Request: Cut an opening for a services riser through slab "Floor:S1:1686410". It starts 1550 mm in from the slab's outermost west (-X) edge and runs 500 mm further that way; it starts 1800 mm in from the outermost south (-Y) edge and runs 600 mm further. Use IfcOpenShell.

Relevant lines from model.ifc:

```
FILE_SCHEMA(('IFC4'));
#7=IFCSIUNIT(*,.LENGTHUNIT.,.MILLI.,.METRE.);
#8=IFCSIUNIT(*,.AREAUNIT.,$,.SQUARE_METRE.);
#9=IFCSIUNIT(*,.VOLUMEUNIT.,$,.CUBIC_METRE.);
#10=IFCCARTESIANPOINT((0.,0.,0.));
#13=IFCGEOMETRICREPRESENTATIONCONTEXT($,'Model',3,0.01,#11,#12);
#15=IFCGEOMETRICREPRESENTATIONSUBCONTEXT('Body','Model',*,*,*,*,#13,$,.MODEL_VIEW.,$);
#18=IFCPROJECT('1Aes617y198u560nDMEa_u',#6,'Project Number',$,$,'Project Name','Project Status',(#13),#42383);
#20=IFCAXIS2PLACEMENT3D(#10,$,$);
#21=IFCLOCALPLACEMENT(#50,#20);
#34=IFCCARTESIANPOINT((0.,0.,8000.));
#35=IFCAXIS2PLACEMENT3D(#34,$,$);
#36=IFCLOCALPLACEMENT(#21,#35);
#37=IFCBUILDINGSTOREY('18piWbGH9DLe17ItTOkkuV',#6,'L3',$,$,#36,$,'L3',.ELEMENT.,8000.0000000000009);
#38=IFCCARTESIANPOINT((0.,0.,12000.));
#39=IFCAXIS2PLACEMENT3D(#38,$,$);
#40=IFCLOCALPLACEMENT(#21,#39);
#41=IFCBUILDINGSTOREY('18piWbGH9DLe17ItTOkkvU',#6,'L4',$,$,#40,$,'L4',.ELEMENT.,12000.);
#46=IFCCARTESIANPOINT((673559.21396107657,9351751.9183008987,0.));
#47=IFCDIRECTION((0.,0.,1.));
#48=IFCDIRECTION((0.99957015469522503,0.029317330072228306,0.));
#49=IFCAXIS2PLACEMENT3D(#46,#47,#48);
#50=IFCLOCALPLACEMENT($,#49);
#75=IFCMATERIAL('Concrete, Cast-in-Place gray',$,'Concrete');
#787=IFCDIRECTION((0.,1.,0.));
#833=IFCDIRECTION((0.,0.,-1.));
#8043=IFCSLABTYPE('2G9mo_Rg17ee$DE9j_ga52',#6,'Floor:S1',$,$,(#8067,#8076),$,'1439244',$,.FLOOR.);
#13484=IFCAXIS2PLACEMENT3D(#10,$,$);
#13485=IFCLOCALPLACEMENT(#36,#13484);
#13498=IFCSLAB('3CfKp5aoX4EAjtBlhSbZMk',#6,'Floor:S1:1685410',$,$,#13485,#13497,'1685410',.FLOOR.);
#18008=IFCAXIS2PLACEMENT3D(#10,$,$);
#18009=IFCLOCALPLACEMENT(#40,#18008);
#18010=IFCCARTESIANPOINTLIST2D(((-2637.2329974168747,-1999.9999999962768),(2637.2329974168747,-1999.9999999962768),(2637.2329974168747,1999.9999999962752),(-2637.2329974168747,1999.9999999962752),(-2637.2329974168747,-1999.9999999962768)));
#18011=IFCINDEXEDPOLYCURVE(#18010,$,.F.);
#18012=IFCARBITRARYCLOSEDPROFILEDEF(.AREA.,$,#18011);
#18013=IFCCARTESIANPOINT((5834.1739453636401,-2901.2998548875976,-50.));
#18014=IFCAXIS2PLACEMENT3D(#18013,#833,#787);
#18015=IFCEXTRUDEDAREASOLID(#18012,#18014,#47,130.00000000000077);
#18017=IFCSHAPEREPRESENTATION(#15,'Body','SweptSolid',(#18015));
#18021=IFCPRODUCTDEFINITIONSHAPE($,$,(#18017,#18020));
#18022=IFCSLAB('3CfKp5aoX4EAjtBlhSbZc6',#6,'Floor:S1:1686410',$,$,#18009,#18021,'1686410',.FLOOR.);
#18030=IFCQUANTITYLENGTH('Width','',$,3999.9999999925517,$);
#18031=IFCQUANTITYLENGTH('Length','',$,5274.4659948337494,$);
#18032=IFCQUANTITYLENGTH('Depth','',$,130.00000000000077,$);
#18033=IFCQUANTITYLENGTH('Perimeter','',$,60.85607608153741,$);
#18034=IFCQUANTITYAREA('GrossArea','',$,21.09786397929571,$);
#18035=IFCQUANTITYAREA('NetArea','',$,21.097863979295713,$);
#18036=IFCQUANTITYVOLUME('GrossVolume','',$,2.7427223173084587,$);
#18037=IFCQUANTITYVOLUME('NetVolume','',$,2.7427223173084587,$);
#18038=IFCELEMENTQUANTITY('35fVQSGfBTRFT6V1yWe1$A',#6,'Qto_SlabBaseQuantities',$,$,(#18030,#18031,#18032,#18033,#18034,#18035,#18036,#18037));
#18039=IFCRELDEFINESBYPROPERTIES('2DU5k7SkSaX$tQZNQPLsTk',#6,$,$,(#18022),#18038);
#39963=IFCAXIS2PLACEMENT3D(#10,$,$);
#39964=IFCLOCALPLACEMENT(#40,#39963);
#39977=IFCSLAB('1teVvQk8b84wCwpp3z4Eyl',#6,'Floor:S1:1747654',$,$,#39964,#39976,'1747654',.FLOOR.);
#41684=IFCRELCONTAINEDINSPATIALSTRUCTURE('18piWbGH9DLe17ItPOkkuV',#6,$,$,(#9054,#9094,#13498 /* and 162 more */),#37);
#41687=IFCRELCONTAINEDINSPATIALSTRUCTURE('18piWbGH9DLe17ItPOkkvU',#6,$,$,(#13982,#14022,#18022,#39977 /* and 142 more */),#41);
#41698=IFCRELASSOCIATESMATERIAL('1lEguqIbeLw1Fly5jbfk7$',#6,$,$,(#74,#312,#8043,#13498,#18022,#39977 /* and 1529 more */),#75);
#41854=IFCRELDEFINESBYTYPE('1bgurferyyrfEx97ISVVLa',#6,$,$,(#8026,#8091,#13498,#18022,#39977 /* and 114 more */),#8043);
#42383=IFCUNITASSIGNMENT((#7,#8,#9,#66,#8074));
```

```python
import numpy as np
import ifcopenshell
import ifcopenshell.api.feature
import ifcopenshell.api.geometry
import ifcopenshell.api.pset
import ifcopenshell.api.root
import ifcopenshell.geom
import ifcopenshell.util.element
import ifcopenshell.util.placement
import ifcopenshell.util.representation
import ifcopenshell.util.shape
import ifcopenshell.util.unit

model = ifcopenshell.open("model.ifc")
unit_scale = ifcopenshell.util.unit.calculate_unit_scale(model)
area_scale = ifcopenshell.util.unit.calculate_unit_scale(model, "AREAUNIT")
volume_scale = ifcopenshell.util.unit.calculate_unit_scale(model, "VOLUMEUNIT")
settings = ifcopenshell.geom.settings()


def volume(element):
    """Net volume in cubic metres, openings subtracted."""
    shape = ifcopenshell.geom.create_shape(settings, element)
    return ifcopenshell.util.shape.get_volume(shape.geometry)


slab = model.by_id(18022)
before = volume(slab)

# Extent in the slab's own axes, in metres. The edges named are its -X and -Y sides.
slab_shape = ifcopenshell.geom.create_shape(settings, slab)
vertices = ifcopenshell.util.shape.get_vertices(slab_shape.geometry)
x_min, y_min, bottom = vertices.min(axis=0)
top = vertices[:, 2].max()

opening = ifcopenshell.api.root.create_entity(model, ifc_class="IfcOpeningElement", name="Services riser opening", predefined_type="OPENING")
context = ifcopenshell.util.representation.get_context(model, "Model", "Body", "MODEL_VIEW")
width, depth = 0.5, 0.6
outline = [(0.0, 0.0), (width, 0.0), (width, depth), (0.0, depth), (0.0, 0.0)]
# Overshoot both faces by 50 mm so the cut is clean.
shape = ifcopenshell.api.geometry.add_slab_representation(
    model, context=context, depth=top - bottom + 0.1, polyline=outline
)
ifcopenshell.api.geometry.assign_representation(model, product=opening, representation=shape)

matrix = ifcopenshell.util.placement.get_local_placement(slab.ObjectPlacement)
matrix[:, 3] = matrix @ np.append(np.array([x_min + 1.55, y_min + 1.8, bottom - 0.05]) / unit_scale, 1.0)
ifcopenshell.api.geometry.edit_object_placement(model, product=opening, matrix=matrix, is_si=False)
ifcopenshell.api.feature.add_feature(model, feature=opening, element=slab)

after = volume(slab)

# Update the slab's stored quantities.
qto = model.by_id(ifcopenshell.util.element.get_pset(slab, "Qto_SlabBaseQuantities", should_inherit=False)["id"])
ifcopenshell.api.pset.edit_qto(model, qto=qto, properties={
    "NetArea": after / (top - bottom) / area_scale,
    "NetVolume": after / volume_scale,
})

print(f"slab volume {before:.3f} -> {after:.3f} m3")

model.write("model_updated.ifc")
```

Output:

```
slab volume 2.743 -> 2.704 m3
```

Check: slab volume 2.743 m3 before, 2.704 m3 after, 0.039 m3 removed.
